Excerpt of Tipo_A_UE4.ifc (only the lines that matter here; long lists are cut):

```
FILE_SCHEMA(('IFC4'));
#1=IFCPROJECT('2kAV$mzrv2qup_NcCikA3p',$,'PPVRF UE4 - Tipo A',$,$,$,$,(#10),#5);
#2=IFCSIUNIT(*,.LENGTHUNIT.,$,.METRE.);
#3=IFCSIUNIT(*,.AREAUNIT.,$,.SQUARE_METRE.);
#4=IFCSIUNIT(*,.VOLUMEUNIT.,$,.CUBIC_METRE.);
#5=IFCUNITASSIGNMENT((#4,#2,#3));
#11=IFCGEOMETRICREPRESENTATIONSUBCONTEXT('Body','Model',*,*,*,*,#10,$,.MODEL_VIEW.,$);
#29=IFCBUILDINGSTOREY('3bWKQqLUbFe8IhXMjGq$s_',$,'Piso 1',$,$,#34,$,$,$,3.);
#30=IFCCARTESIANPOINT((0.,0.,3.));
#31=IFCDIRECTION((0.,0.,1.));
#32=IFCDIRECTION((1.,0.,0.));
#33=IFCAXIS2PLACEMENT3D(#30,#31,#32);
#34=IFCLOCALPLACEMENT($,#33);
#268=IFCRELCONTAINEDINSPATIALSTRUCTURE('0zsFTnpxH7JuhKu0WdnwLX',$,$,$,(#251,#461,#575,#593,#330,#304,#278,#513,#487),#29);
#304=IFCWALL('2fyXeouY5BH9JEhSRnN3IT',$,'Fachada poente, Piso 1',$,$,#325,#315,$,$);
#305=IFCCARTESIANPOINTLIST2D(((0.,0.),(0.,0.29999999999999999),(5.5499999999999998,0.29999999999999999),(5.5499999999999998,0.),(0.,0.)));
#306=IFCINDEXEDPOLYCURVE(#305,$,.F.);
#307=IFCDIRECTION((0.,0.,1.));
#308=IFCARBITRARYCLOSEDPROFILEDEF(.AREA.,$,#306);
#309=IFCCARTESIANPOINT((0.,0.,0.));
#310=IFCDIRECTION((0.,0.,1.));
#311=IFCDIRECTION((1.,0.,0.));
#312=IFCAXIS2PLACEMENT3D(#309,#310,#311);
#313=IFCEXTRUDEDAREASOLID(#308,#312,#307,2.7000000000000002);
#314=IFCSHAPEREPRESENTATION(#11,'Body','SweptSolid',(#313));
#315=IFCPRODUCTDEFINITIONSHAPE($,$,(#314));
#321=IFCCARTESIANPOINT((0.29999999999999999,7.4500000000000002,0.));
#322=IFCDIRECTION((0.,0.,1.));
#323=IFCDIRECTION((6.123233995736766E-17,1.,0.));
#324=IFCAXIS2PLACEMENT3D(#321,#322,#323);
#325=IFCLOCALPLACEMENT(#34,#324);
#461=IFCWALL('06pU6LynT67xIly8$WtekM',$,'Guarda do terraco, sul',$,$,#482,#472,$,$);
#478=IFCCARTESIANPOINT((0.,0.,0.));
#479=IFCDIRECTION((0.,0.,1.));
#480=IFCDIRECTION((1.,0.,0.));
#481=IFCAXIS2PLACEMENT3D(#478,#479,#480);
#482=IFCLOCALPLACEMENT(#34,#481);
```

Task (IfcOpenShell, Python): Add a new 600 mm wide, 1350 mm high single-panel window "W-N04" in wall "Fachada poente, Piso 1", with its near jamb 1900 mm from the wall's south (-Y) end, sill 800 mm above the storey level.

```python
import numpy as np
import ifcopenshell
import ifcopenshell.api.feature
import ifcopenshell.api.geometry
import ifcopenshell.api.root
import ifcopenshell.api.spatial
import ifcopenshell.geom
import ifcopenshell.util.element
import ifcopenshell.util.placement
import ifcopenshell.util.representation
import ifcopenshell.util.shape
import ifcopenshell.util.unit

model = ifcopenshell.open("Tipo_A_UE4.ifc")
unit_scale = ifcopenshell.util.unit.calculate_unit_scale(model)
settings = ifcopenshell.geom.settings()


def volume(element):
    """Net volume in cubic metres, openings subtracted."""
    shape = ifcopenshell.geom.create_shape(settings, element)
    return ifcopenshell.util.shape.get_volume(shape.geometry)


wall = model.by_guid("2fyXeouY5BH9JEhSRnN3IT")
storey = ifcopenshell.util.element.get_container(wall, ifc_class="IfcBuildingStorey")
context = ifcopenshell.util.representation.get_context(model, "Model", "Body", "MODEL_VIEW")
before = volume(wall)

width, height, from_end, sill = 0.6, 1.35, 1.9, 0.8  # metres

# The wall runs along its own X axis, and the end named is its -X end.
wall_shape = ifcopenshell.geom.create_shape(settings, wall)
x, y, z = ifcopenshell.util.shape.get_vertices(wall_shape.geometry).T
start = x.min() + from_end
face, thickness = float(y.min()), float(y.max() - y.min())
wall_matrix = ifcopenshell.util.placement.get_local_placement(wall.ObjectPlacement)
level = ifcopenshell.util.placement.get_local_placement(storey.ObjectPlacement)[2, 3]


def in_wall(x, y):
    """Placement at x, y metres in the wall's axes, at sill height."""
    matrix = wall_matrix.copy()
    matrix[:, 3] = wall_matrix @ np.array([x / unit_scale, y / unit_scale, 0.0, 1.0])
    matrix[2, 3] = level + sill / unit_scale
    return matrix


# Opening: a box that overshoots both wall faces by 50 mm.
opening = ifcopenshell.api.root.create_entity(model, ifc_class="IfcOpeningElement", predefined_type="OPENING")
box = ifcopenshell.api.geometry.add_wall_representation(
    model, context=context, length=width, height=height, thickness=thickness + 0.1
)
ifcopenshell.api.geometry.assign_representation(model, product=opening, representation=box)
ifcopenshell.api.geometry.edit_object_placement(model, product=opening, matrix=in_wall(start, face - 0.05), is_si=False)
ifcopenshell.api.feature.add_feature(model, feature=opening, element=wall)

window = ifcopenshell.api.root.create_entity(model, ifc_class="IfcWindow", name="W-N04", predefined_type="WINDOW")
window.OverallWidth, window.OverallHeight = width / unit_scale, height / unit_scale
window.PartitioningType = "SINGLE_PANEL"
body = ifcopenshell.api.geometry.add_window_representation(
    model,
    context=context,
    overall_width=window.OverallWidth,
    overall_height=window.OverallHeight,
    partition_type="SINGLE_PANEL",
)
ifcopenshell.api.geometry.assign_representation(model, product=window, representation=body)
ifcopenshell.api.spatial.assign_container(model, products=[window], relating_structure=storey)
ifcopenshell.api.feature.add_filling(model, opening=opening, element=window)

# Centre the window in the wall's thickness.
ifcopenshell.api.geometry.edit_object_placement(model, product=window, matrix=in_wall(start, face), is_si=False)
window_shape = ifcopenshell.geom.create_shape(settings, window)
depth = ifcopenshell.util.shape.get_vertices(window_shape.geometry)[:, 1]
offset = face + thickness / 2 - (depth.min() + depth.max()) / 2
ifcopenshell.api.geometry.edit_object_placement(model, product=window, matrix=in_wall(start, offset), is_si=False)

after = volume(wall)

print(f"wall volume {before:.3f} -> {after:.3f} m3")

model.write("Tipo_A_UE4_updated.ifc")
```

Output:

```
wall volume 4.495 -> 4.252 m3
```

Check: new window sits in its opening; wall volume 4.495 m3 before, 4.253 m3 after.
